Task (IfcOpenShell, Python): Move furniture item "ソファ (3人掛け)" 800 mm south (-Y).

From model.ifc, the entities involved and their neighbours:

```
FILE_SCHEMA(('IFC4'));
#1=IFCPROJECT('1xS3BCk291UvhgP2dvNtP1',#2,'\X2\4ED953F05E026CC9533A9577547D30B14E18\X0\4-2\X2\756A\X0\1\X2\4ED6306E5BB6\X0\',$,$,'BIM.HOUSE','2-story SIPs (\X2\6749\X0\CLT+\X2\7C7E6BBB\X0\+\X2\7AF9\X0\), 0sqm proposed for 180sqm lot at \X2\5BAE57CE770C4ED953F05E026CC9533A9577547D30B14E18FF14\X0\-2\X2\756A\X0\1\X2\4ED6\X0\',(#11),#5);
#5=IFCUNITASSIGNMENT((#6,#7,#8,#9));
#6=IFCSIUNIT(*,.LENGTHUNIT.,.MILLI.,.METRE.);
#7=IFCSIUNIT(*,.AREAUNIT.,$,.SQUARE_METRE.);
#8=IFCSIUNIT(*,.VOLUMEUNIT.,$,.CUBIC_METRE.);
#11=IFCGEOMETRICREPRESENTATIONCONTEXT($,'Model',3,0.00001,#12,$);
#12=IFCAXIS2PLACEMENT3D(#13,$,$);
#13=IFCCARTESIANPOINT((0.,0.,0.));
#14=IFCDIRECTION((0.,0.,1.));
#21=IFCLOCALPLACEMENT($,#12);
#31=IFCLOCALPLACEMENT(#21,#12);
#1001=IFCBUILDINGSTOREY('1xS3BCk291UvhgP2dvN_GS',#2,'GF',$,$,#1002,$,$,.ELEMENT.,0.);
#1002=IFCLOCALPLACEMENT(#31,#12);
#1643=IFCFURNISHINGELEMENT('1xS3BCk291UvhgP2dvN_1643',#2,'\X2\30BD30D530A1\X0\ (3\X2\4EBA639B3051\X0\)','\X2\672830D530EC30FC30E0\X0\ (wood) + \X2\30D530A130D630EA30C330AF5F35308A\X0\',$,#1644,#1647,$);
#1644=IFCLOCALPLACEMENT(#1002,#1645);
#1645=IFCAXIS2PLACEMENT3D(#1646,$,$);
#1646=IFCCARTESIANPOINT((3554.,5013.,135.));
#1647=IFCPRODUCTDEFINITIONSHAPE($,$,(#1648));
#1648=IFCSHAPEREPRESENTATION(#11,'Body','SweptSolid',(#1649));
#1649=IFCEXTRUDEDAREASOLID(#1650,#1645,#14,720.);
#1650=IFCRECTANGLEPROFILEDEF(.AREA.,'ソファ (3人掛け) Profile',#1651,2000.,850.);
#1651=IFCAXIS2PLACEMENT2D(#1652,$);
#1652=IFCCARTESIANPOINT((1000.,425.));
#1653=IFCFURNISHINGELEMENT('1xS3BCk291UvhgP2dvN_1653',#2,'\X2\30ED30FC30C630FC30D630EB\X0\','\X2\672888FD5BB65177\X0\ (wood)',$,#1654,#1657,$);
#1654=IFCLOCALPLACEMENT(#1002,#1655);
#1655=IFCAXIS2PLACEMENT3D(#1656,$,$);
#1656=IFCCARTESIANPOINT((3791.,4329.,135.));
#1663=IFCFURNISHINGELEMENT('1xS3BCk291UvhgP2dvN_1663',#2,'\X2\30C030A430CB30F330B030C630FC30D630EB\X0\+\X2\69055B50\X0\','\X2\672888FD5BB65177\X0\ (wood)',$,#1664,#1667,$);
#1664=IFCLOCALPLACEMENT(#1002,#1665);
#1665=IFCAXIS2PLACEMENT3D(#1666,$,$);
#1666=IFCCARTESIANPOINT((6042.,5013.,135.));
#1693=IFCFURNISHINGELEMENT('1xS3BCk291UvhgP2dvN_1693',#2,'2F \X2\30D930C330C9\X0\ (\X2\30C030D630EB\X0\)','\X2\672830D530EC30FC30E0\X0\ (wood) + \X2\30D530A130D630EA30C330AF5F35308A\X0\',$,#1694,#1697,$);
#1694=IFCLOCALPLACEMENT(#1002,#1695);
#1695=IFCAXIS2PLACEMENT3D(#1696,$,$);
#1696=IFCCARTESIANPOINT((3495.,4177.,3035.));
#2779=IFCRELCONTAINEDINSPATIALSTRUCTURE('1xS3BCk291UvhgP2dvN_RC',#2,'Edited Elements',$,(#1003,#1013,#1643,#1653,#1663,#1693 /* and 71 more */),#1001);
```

```python
import ifcopenshell
import ifcopenshell.api.geometry
import ifcopenshell.util.placement
import ifcopenshell.util.unit

model = ifcopenshell.open("model.ifc")
unit_scale = ifcopenshell.util.unit.calculate_unit_scale(model)

item = model.by_guid("1xS3BCk291UvhgP2dvN_1643")
matrix = ifcopenshell.util.placement.get_local_placement(item.ObjectPlacement)
matrix[1, 3] -= 0.8 / unit_scale
ifcopenshell.api.geometry.edit_object_placement(model, product=item, matrix=matrix, is_si=False)

print(ifcopenshell.util.placement.get_local_placement(item.ObjectPlacement).round(3) + 0.0)

model.write("model_updated.ifc")
```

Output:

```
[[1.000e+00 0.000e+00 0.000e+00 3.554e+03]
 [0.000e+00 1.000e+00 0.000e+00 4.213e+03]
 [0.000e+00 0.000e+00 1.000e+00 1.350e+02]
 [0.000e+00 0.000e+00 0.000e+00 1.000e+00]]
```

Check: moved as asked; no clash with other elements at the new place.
